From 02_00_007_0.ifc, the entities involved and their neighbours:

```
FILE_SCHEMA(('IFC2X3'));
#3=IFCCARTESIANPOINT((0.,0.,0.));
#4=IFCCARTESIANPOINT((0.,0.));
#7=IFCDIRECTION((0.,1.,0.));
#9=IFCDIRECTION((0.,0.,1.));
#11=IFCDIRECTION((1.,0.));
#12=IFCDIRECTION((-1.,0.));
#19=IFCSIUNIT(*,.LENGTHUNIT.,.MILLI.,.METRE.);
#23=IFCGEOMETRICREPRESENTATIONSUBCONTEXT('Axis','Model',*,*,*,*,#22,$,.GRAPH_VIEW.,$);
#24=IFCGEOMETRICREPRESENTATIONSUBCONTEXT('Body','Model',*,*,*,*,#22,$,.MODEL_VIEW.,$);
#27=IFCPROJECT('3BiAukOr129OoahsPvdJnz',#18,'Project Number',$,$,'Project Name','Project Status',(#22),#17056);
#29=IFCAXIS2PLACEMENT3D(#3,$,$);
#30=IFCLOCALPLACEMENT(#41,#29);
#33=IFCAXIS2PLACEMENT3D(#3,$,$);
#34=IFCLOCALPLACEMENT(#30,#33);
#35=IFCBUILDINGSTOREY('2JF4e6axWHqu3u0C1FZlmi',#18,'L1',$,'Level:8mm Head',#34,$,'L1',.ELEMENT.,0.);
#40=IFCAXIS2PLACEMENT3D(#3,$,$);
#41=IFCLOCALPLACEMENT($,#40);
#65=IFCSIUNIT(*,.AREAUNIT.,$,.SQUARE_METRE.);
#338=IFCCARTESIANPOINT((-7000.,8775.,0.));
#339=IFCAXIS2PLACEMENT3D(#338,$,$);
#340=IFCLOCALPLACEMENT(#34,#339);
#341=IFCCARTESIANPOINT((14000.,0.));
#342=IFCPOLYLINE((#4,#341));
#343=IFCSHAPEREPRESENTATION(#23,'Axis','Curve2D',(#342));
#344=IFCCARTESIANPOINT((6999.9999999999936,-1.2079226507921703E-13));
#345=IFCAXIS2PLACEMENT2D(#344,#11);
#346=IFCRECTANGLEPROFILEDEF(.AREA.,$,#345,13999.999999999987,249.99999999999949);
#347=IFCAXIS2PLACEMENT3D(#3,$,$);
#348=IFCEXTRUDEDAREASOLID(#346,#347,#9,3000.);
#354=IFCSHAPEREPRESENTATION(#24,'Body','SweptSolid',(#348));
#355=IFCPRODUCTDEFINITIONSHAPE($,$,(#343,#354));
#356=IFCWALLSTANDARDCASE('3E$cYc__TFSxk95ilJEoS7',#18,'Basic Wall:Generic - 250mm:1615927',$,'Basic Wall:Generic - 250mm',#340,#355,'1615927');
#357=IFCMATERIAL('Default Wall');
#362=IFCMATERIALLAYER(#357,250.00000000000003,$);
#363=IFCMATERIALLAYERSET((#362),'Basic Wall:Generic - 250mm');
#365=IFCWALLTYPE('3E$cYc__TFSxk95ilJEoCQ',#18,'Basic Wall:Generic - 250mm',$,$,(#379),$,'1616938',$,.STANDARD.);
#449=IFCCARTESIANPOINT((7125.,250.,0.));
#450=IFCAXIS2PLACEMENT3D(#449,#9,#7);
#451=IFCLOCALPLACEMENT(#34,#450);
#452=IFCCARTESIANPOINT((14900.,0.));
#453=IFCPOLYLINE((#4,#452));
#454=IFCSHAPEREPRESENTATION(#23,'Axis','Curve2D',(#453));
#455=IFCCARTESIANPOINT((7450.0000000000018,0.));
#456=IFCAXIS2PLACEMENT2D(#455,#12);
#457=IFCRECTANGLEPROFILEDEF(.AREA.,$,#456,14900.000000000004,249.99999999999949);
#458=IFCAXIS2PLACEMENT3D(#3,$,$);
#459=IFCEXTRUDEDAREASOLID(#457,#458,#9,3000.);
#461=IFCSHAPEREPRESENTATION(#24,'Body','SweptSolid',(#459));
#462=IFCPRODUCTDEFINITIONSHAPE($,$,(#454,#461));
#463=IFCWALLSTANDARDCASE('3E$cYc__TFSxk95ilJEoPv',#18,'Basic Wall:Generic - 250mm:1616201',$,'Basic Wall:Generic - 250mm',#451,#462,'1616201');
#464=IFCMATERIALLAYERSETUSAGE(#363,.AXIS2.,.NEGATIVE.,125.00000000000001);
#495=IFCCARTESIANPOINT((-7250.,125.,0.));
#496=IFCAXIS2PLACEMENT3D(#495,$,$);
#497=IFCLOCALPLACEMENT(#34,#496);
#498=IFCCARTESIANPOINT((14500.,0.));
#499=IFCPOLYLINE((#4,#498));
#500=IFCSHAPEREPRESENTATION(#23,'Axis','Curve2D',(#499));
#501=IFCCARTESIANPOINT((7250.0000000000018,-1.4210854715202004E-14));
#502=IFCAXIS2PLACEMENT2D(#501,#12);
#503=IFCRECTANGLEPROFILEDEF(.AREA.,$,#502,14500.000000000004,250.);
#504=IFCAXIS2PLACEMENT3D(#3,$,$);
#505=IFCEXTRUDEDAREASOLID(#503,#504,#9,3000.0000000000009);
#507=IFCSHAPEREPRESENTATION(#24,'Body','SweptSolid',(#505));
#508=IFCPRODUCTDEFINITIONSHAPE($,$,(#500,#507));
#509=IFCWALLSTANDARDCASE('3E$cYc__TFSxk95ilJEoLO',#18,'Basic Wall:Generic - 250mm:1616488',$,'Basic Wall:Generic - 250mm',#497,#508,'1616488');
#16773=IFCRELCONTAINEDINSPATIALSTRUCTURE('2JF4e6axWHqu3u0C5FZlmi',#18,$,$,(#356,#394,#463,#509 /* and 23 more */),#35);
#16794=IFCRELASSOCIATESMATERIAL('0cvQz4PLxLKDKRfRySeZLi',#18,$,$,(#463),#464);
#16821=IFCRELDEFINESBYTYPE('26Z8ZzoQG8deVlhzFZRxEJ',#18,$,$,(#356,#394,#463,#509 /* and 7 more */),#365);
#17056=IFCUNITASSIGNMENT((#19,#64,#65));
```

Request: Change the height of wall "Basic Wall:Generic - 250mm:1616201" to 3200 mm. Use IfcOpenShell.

```python
import ifcopenshell
import ifcopenshell.geom
import ifcopenshell.util.representation
import ifcopenshell.util.shape

model = ifcopenshell.open("02_00_007_0.ifc")
settings = ifcopenshell.geom.settings()


def volume(element):
    """Net volume in cubic metres, openings subtracted."""
    shape = ifcopenshell.geom.create_shape(settings, element)
    return ifcopenshell.util.shape.get_volume(shape.geometry)


wall = model.by_guid("3E$cYc__TFSxk95ilJEoPv")
before = volume(wall)

body = ifcopenshell.util.representation.get_representation(wall, "Model", "Body")
solid = body.Items[0]
old_height = solid.Depth
solid.Depth = 3200.0
after = volume(wall)

print(f"height {old_height:g} -> {solid.Depth:g}, volume {before:.3f} -> {after:.3f} m3")

model.write("02_00_007_0_rev.ifc")
```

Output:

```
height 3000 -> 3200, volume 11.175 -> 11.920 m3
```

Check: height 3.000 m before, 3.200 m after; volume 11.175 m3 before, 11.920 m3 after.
